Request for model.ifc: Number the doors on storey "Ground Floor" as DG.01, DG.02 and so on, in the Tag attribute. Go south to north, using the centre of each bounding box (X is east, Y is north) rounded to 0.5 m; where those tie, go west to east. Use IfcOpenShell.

First a look at what the model holds.

```python
import ifcopenshell
import ifcopenshell.util.element
import ifcopenshell.util.placement

model = ifcopenshell.open("model.ifc")
print(model.schema)
storey = next(s for s in model.by_type("IfcBuildingStorey") if s.Name == "Ground Floor")
doors = [e for e in ifcopenshell.util.element.get_decomposition(storey) if e.is_a("IfcDoor")]
for e in sorted(doors, key=lambda e: e.id()):
    origin = ifcopenshell.util.placement.get_local_placement(e.ObjectPlacement)[:3, 3]
    print(e.id(), e.Tag, e.Name, origin.round(2) + 0.0, sep=" | ")
```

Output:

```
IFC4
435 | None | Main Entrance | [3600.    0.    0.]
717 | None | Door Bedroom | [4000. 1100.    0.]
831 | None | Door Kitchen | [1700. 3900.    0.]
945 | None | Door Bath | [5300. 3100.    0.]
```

```python
import ifcopenshell
import ifcopenshell.geom
import ifcopenshell.util.element
import ifcopenshell.util.shape

model = ifcopenshell.open("model.ifc")
settings = ifcopenshell.geom.settings()
settings.set("use-world-coords", True)


def centre(element):
    shape = ifcopenshell.geom.create_shape(settings, element)
    return ifcopenshell.util.shape.get_bbox_centroid(shape.geometry)


storey = next(s for s in model.by_type("IfcBuildingStorey") if s.Name == "Ground Floor")
doors = [e for e in ifcopenshell.util.element.get_decomposition(storey) if e.is_a("IfcDoor")]

# Insertion points can sit at a corner or the storey origin, so sort by the geometry (in metres).
centres = {e: centre(e) for e in doors}
doors.sort(key=lambda e: (round(centres[e][1] / 0.5), centres[e][0]))

for i, e in enumerate(doors, start=1):
    number = f"DG.{i:02d}"
    e.Tag = number
    print(e.id(), number)

model.write("model_v2.ifc")
```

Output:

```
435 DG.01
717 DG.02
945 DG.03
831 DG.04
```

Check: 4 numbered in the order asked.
